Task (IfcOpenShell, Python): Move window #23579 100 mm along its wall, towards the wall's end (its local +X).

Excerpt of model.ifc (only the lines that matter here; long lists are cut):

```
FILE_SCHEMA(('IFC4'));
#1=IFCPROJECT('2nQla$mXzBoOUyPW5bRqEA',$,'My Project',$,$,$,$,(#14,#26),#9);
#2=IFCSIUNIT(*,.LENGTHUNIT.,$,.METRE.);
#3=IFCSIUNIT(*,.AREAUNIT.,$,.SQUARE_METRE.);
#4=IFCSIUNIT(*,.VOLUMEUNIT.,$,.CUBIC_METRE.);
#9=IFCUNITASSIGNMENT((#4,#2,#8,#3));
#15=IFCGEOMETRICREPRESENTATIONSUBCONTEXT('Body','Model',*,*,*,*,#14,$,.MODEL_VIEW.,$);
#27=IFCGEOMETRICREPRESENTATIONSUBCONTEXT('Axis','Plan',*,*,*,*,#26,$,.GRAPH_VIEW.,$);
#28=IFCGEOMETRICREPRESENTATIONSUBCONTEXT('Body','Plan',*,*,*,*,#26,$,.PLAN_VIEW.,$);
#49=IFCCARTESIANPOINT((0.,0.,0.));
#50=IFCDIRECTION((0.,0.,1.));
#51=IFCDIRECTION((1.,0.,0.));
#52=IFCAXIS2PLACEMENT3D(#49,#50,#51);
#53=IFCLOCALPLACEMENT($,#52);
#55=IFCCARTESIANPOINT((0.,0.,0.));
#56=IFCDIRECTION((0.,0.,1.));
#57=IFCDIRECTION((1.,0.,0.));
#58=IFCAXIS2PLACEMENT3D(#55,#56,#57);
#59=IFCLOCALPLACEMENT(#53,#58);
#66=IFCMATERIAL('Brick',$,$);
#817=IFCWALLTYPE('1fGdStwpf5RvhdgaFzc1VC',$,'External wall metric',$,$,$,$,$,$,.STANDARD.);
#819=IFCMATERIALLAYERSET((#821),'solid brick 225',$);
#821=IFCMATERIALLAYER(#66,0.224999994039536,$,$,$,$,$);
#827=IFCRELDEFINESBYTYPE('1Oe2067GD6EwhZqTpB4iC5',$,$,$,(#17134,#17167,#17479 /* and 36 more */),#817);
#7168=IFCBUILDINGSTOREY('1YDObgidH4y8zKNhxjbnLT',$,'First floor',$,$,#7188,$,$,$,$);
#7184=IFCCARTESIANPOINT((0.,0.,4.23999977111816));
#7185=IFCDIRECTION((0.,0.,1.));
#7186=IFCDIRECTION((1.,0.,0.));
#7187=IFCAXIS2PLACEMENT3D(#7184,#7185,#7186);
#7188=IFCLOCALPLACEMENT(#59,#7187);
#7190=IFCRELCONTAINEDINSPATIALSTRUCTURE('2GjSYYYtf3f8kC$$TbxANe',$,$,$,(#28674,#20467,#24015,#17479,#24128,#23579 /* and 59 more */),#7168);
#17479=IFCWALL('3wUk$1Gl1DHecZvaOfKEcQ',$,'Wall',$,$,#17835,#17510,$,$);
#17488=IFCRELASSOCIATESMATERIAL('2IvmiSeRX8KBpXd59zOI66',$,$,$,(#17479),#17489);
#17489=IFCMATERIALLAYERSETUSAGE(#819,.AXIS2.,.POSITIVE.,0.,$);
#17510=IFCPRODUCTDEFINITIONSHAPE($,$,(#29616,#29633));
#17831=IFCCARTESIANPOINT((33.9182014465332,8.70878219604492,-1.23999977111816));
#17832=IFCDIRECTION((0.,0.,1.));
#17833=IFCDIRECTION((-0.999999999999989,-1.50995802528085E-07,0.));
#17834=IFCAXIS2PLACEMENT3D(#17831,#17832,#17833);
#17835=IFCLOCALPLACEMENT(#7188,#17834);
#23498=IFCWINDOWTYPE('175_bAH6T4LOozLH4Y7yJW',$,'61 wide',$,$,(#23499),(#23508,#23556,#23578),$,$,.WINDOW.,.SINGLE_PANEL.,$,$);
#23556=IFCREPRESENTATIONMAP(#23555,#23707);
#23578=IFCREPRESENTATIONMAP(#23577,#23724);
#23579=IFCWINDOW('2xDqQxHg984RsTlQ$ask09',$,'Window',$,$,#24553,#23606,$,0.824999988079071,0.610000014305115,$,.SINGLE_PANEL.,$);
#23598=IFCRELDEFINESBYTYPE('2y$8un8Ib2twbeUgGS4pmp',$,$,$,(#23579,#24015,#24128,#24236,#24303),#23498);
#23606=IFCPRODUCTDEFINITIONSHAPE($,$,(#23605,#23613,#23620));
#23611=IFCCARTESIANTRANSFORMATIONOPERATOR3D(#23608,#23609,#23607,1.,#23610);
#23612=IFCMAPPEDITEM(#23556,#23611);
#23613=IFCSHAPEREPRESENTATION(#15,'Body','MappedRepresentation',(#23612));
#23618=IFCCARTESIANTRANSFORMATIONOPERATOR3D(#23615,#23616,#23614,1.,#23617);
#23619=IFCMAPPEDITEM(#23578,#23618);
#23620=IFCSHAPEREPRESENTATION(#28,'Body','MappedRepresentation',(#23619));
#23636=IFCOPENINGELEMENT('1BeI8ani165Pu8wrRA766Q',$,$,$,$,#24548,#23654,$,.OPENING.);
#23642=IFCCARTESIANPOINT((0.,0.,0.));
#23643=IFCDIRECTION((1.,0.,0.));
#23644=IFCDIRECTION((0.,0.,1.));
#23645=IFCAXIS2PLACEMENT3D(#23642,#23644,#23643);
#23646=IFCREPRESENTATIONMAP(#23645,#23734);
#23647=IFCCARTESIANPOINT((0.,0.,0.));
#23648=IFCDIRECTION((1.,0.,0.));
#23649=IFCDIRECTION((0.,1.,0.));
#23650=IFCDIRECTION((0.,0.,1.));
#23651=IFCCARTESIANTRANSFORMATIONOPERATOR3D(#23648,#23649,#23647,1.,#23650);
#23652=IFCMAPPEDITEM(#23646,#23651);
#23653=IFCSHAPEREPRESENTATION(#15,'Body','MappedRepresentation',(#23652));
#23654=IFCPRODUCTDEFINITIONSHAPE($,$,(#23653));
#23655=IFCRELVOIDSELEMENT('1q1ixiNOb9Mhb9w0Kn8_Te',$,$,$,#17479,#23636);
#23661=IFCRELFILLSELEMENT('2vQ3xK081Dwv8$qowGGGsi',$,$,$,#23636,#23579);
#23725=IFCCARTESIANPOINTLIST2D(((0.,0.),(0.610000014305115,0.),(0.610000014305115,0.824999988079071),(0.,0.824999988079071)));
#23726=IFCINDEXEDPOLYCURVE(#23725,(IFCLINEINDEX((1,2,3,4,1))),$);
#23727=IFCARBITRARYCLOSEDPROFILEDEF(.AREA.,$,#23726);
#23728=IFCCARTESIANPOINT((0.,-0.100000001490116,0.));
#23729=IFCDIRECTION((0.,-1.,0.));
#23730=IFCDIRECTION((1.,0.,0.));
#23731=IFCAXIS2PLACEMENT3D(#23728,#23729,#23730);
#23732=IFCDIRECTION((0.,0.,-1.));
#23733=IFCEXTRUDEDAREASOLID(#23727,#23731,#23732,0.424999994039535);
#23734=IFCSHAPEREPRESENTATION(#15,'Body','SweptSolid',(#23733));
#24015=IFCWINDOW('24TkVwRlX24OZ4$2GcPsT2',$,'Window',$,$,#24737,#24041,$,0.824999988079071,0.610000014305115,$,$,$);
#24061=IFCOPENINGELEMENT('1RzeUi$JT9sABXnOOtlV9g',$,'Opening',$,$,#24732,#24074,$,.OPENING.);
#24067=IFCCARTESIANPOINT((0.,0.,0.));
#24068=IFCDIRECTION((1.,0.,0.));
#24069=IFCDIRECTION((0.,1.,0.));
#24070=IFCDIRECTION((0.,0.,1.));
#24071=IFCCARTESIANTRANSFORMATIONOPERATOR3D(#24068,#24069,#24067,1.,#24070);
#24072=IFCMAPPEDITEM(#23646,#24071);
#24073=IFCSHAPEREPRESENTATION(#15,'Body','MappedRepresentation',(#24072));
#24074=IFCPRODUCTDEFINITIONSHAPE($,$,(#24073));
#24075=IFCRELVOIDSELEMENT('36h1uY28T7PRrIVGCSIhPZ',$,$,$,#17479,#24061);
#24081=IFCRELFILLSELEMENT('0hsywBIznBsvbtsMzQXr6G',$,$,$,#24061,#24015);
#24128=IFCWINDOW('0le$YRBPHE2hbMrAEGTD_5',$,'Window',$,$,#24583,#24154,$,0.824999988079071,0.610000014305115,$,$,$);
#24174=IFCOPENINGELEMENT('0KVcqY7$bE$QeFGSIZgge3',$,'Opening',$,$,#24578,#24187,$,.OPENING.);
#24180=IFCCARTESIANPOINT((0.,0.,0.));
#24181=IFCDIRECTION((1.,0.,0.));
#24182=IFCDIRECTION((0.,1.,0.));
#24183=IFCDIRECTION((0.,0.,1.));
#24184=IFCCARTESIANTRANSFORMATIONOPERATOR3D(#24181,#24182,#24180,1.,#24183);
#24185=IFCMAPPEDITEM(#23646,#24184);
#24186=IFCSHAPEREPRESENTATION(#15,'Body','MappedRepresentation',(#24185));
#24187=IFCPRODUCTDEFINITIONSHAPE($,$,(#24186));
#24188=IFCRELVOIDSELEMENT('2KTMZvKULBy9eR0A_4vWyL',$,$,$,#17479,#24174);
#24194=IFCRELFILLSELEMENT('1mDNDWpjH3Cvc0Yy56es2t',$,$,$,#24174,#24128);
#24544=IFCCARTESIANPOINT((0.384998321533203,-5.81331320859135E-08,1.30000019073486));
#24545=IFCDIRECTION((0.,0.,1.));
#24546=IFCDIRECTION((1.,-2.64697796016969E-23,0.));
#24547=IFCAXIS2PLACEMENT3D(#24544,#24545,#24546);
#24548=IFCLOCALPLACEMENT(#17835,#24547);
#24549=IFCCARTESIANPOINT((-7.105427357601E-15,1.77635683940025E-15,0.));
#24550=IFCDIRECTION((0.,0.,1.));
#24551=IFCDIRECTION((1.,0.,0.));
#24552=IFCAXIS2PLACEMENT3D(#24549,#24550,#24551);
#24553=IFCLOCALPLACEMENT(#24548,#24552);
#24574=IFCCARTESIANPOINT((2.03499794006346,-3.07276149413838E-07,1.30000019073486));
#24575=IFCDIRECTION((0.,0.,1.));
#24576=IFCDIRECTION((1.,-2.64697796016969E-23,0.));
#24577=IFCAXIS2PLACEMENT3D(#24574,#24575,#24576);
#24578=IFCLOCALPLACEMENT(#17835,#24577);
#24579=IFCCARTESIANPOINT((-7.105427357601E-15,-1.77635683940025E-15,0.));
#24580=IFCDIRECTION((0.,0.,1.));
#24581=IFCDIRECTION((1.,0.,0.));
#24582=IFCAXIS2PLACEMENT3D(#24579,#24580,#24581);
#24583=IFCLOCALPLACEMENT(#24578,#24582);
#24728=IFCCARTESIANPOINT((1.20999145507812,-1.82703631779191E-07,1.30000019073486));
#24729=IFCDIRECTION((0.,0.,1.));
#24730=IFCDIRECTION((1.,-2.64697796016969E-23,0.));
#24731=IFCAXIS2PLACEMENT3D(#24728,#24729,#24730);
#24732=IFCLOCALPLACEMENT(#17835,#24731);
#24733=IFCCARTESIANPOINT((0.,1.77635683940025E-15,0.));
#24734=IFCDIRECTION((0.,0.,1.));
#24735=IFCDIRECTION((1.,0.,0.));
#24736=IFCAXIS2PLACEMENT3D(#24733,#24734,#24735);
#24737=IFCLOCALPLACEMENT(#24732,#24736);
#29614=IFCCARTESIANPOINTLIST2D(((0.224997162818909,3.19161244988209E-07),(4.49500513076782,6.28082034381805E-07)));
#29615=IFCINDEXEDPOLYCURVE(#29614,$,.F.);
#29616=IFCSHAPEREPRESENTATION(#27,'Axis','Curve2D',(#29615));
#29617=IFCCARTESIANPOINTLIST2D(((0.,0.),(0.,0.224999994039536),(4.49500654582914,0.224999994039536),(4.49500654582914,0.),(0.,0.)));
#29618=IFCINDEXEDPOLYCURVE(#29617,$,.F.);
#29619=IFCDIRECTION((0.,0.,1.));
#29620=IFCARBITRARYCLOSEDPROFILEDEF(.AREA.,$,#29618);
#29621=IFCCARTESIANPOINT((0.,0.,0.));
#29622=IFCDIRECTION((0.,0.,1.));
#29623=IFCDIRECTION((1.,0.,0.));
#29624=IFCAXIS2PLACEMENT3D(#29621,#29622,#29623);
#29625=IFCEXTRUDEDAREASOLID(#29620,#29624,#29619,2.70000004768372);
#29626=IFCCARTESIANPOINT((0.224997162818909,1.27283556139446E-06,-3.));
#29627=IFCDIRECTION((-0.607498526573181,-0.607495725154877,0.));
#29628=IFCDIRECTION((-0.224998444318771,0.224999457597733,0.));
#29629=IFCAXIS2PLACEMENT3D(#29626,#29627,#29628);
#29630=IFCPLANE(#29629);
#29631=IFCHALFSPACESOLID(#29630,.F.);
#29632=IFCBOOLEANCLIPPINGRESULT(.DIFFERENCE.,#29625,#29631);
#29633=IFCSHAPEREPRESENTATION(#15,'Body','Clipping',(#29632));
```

```python
import ifcopenshell
import ifcopenshell.api.geometry
import ifcopenshell.util.placement
import ifcopenshell.util.unit

model = ifcopenshell.open("model.ifc")
unit_scale = ifcopenshell.util.unit.calculate_unit_scale(model)

window = model.by_guid("2xDqQxHg984RsTlQ$ask09")
opening = window.FillsVoids[0].RelatingOpeningElement
wall = opening.VoidsElements[0].RelatingBuildingElement

wall_matrix = ifcopenshell.util.placement.get_local_placement(wall.ObjectPlacement)
shift = wall_matrix[:3, 0] * 0.1 / unit_scale
before = ifcopenshell.util.placement.get_local_placement(window.ObjectPlacement)[:3, 3].copy()

# The window is placed relative to its opening, so it follows when the opening moves.
matrix = ifcopenshell.util.placement.get_local_placement(opening.ObjectPlacement)
matrix[:3, 3] += shift
ifcopenshell.api.geometry.edit_object_placement(
    model, product=opening, matrix=matrix, is_si=False, should_transform_children=True
)

after = ifcopenshell.util.placement.get_local_placement(window.ObjectPlacement)[:3, 3]
print("window moved by", (after - before).round(3) + 0.0)

model.write("model_v2.ifc")
```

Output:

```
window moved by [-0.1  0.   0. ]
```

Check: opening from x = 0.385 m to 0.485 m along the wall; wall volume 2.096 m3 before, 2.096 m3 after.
